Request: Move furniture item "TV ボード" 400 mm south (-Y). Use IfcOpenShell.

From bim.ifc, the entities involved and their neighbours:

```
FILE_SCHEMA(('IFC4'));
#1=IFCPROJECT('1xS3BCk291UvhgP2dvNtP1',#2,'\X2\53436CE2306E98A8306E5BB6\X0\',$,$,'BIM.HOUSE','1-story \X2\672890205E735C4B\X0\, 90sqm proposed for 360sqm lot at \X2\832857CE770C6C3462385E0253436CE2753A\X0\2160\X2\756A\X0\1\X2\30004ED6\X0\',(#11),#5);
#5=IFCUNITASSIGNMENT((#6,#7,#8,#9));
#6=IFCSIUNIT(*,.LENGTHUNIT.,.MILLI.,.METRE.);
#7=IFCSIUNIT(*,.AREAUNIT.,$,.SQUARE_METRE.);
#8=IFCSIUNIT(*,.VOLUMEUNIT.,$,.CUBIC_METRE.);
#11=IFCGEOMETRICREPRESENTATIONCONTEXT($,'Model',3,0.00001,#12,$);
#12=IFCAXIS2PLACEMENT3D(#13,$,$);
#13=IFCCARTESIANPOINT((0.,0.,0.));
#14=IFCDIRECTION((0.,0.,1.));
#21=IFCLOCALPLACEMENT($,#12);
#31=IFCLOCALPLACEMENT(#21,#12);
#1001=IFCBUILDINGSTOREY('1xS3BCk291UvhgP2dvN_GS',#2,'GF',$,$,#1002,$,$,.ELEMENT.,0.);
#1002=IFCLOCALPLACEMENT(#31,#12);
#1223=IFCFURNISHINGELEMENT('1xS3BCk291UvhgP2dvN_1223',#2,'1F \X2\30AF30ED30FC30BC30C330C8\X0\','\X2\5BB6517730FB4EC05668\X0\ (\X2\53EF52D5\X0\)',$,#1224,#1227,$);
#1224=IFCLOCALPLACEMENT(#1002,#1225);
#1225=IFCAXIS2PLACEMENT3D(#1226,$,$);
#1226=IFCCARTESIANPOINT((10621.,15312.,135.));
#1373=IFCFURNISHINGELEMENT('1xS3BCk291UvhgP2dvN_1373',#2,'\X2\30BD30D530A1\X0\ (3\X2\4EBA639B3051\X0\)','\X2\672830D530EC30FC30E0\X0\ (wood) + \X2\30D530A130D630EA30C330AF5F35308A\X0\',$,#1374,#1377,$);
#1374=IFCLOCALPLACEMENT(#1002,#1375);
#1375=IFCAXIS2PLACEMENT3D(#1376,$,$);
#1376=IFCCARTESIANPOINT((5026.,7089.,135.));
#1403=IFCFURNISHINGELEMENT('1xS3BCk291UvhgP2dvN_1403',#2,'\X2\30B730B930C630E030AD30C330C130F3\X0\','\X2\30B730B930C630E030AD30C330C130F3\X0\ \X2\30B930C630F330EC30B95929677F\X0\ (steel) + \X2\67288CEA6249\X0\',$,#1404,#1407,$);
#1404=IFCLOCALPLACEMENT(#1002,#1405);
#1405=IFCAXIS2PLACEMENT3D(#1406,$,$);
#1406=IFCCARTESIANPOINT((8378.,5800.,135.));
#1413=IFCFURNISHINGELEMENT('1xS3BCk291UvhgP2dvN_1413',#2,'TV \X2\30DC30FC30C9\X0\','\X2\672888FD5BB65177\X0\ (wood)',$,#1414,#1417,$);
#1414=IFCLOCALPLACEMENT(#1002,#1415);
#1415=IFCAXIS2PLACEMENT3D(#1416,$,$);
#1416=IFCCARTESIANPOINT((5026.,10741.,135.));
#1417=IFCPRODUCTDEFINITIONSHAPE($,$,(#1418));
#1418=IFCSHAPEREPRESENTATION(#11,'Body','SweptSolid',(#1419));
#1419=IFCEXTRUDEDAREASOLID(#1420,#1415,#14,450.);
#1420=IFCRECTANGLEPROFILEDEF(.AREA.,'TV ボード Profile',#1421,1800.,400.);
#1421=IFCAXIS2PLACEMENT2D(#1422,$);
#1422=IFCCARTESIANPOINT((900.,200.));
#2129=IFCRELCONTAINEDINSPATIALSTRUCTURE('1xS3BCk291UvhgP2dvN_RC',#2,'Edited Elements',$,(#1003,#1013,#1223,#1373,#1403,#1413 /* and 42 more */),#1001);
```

```python
import ifcopenshell
import ifcopenshell.api.geometry
import ifcopenshell.util.placement
import ifcopenshell.util.unit

model = ifcopenshell.open("bim.ifc")
unit_scale = ifcopenshell.util.unit.calculate_unit_scale(model)

item = model.by_id(1413)
matrix = ifcopenshell.util.placement.get_local_placement(item.ObjectPlacement)
matrix[1, 3] -= 0.4 / unit_scale
ifcopenshell.api.geometry.edit_object_placement(model, product=item, matrix=matrix, is_si=False)

print(ifcopenshell.util.placement.get_local_placement(item.ObjectPlacement).round(3) + 0.0)

model.write("bim_edited.ifc")
```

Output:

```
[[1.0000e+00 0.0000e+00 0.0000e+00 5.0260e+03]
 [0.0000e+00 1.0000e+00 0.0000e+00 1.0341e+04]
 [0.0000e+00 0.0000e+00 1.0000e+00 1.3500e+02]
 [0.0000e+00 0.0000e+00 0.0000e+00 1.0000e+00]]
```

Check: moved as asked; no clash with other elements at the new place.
